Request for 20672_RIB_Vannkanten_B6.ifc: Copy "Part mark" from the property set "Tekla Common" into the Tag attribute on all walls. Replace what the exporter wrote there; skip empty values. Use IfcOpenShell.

First a look at what the model holds.

```python
import ifcopenshell
import ifcopenshell.util.element

model = ifcopenshell.open("20672_RIB_Vannkanten_B6.ifc")
print(model.schema)
walls = model.by_type("IfcWall")
print(len(walls), "walls")
for e in walls[:8]:
    source = ifcopenshell.util.element.get_pset(e, "Tekla Common", "Part mark")
    target = e.Tag
    print(e.id(), repr(source), repr(target), sep=" | ")
```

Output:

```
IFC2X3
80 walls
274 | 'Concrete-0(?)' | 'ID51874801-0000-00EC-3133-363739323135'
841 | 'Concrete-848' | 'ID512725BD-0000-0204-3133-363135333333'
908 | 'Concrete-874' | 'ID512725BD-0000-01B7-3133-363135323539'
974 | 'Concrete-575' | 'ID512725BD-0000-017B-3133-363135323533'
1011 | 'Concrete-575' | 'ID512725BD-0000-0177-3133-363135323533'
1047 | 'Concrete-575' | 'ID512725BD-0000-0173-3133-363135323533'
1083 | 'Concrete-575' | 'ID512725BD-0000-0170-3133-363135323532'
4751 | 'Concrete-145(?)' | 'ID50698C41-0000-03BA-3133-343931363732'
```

```python
import ifcopenshell
import ifcopenshell.util.element

model = ifcopenshell.open("20672_RIB_Vannkanten_B6.ifc")

count = 0
for e in model.by_type("IfcWall"):
    value = ifcopenshell.util.element.get_pset(e, "Tekla Common", "Part mark")
    current = e.Tag
    if not value or not value.strip() or current == value:
        continue
    e.Tag = value
    count += 1

print(count, "walls updated")

model.write("20672_RIB_Vannkanten_B6-out.ifc")
```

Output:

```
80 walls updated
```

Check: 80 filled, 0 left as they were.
